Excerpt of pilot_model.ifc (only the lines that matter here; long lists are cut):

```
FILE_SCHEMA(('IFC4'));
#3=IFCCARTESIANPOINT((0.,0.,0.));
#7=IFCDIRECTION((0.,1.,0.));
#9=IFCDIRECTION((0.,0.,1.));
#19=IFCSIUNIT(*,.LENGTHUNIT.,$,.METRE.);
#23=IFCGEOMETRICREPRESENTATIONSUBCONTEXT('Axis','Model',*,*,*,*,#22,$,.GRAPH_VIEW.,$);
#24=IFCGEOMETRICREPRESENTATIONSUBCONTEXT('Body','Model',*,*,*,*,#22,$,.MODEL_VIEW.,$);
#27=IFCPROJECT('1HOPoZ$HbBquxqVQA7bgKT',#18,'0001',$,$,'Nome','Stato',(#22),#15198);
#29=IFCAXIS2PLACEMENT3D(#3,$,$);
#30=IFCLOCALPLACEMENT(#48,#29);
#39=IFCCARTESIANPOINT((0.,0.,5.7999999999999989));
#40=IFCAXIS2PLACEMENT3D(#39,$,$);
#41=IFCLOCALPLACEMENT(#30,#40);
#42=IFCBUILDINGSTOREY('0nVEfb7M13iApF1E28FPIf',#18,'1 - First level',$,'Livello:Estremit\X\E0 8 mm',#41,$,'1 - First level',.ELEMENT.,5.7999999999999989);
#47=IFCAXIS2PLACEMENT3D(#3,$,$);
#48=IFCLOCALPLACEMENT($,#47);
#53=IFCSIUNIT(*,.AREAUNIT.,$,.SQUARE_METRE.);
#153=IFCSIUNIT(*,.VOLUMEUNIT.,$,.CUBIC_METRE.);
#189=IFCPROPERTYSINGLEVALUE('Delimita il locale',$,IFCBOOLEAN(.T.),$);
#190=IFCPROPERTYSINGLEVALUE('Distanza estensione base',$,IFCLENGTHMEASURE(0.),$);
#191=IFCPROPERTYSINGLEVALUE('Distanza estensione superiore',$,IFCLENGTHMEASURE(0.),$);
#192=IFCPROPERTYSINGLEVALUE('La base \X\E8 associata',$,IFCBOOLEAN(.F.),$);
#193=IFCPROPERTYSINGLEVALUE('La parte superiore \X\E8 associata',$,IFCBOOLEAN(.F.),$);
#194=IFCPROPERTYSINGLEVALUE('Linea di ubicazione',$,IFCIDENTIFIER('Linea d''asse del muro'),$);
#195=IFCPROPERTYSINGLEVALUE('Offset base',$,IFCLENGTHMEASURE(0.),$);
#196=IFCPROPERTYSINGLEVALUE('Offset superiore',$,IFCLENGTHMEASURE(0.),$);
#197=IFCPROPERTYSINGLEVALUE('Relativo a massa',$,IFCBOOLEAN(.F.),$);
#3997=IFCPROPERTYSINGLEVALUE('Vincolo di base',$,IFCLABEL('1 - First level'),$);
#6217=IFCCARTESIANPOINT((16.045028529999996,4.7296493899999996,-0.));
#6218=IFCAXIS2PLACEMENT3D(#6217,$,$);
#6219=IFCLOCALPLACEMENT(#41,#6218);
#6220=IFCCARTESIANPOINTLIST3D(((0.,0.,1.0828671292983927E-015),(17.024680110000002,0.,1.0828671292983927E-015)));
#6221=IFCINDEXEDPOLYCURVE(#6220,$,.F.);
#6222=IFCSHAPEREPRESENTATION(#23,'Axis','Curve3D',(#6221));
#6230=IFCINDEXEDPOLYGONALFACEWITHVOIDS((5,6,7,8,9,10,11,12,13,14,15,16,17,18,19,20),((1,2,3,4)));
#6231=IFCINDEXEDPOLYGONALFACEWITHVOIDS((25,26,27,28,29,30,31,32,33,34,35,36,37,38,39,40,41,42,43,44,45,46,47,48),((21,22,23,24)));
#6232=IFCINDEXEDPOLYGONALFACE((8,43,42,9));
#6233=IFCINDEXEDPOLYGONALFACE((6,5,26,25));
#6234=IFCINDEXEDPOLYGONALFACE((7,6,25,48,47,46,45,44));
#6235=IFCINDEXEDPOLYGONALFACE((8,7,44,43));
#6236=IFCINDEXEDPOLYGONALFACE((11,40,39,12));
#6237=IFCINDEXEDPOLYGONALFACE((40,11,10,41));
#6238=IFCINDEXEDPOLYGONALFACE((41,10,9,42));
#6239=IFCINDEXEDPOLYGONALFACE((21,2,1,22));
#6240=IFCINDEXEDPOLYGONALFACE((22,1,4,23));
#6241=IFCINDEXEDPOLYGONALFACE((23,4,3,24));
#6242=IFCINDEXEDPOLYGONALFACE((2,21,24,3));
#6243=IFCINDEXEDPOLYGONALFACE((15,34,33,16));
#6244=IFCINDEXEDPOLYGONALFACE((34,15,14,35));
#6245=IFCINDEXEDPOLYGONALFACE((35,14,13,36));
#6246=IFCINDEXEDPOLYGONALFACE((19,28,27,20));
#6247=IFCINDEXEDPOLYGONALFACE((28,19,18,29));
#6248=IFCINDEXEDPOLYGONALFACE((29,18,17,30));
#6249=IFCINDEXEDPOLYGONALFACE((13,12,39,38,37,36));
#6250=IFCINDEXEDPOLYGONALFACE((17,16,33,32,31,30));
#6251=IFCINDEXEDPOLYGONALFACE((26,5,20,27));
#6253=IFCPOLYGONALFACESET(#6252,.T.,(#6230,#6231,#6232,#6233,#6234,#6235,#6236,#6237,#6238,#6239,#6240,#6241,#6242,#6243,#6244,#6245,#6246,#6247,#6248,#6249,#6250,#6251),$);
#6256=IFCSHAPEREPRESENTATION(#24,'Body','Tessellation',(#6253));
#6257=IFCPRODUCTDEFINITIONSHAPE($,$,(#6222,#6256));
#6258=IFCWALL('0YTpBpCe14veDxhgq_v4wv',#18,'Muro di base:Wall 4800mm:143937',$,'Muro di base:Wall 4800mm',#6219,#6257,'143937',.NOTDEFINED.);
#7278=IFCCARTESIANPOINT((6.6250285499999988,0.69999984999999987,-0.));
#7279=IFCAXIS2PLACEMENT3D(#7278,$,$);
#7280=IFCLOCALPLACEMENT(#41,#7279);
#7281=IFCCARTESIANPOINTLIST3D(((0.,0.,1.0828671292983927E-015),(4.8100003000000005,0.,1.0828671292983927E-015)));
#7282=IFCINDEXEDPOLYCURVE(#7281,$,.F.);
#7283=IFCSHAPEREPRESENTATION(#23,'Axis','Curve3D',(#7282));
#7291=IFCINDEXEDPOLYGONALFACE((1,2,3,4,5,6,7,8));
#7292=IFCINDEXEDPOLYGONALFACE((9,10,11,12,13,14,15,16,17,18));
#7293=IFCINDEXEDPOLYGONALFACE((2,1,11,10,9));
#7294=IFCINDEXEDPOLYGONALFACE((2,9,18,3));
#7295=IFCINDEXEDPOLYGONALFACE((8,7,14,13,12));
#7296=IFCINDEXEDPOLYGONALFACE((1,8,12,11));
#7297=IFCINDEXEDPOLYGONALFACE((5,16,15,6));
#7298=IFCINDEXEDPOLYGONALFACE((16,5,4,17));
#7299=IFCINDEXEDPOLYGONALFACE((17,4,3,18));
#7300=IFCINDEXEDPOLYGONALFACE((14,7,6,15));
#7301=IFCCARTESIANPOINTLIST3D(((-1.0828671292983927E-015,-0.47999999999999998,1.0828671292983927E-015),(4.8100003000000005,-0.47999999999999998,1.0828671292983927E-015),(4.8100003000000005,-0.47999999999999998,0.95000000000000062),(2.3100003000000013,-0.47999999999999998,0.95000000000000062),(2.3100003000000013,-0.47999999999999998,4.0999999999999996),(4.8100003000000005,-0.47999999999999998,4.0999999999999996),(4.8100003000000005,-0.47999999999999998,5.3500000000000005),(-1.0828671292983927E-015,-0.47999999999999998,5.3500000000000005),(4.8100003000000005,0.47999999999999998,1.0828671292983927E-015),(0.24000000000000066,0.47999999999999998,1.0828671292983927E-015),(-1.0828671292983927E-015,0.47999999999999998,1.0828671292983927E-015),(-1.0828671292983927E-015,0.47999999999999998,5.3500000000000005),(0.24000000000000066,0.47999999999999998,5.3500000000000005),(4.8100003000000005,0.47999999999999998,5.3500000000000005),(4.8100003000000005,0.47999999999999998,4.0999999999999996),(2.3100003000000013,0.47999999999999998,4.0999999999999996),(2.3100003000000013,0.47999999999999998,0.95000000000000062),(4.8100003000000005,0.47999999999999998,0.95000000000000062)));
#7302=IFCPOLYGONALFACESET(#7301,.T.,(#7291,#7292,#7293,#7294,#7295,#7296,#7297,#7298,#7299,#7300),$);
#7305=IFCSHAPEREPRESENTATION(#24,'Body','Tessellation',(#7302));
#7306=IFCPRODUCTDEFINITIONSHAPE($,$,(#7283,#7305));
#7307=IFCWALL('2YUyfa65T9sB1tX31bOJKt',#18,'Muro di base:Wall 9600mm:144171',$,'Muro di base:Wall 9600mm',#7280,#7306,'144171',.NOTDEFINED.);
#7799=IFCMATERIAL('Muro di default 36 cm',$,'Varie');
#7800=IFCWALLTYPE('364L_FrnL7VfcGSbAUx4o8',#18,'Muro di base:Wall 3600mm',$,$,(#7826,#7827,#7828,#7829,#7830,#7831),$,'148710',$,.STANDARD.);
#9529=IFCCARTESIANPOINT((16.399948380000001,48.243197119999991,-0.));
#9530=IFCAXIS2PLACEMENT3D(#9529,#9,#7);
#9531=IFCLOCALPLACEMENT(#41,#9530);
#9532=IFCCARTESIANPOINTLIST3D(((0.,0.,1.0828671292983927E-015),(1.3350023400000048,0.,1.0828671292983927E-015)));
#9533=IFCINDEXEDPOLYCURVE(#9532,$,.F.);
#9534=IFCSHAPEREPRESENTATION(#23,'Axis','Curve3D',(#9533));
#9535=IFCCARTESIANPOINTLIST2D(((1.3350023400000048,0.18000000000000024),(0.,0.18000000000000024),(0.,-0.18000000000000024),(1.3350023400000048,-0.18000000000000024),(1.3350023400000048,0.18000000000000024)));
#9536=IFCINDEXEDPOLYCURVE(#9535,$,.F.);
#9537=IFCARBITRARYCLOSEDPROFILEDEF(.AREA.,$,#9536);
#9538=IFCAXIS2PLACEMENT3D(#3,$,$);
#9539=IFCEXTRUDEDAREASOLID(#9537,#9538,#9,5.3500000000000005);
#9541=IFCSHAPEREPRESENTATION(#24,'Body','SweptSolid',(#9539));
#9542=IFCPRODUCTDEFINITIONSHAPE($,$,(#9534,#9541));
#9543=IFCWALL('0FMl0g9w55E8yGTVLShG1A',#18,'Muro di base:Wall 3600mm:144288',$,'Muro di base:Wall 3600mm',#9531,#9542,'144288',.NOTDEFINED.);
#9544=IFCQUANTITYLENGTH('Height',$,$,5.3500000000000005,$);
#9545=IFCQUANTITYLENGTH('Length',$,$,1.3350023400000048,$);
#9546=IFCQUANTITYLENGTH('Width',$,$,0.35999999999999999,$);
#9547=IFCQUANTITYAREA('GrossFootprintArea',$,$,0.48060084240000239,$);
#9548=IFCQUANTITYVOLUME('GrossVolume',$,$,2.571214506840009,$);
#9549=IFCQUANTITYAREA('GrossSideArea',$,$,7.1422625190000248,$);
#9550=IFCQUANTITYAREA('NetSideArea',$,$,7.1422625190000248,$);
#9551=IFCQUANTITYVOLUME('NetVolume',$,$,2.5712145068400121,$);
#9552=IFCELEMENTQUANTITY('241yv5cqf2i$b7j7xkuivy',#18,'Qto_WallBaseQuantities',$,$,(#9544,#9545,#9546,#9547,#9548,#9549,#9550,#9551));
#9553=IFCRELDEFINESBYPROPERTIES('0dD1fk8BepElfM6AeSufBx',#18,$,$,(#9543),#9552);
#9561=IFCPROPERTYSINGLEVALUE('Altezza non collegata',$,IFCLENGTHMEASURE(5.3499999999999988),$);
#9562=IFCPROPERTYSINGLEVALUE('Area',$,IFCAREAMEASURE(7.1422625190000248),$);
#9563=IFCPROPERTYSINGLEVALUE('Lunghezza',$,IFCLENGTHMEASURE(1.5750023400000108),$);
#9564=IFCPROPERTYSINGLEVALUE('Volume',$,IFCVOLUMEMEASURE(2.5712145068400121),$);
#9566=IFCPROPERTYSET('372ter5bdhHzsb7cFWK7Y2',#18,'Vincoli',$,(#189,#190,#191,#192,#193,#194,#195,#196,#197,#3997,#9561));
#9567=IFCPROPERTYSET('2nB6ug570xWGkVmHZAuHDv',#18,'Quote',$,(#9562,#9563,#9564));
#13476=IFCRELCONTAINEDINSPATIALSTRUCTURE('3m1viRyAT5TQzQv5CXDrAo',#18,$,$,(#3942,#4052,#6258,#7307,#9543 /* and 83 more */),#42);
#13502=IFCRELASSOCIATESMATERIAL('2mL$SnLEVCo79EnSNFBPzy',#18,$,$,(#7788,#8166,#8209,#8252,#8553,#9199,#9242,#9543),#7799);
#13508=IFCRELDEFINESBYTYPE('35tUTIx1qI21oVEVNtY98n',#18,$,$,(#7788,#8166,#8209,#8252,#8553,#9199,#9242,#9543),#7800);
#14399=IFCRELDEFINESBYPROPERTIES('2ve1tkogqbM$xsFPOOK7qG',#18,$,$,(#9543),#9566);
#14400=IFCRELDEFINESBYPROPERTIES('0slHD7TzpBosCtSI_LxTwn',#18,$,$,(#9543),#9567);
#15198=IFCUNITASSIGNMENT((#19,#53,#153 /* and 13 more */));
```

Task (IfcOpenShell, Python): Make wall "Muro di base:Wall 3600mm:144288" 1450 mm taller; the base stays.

```python
import ifcopenshell
import ifcopenshell.api.pset
import ifcopenshell.geom
import ifcopenshell.util.element
import ifcopenshell.util.representation
import ifcopenshell.util.shape
import ifcopenshell.util.unit

model = ifcopenshell.open("pilot_model.ifc")
unit_scale = ifcopenshell.util.unit.calculate_unit_scale(model)
area_scale = ifcopenshell.util.unit.calculate_unit_scale(model, "AREAUNIT")
volume_scale = ifcopenshell.util.unit.calculate_unit_scale(model, "VOLUMEUNIT")
settings = ifcopenshell.geom.settings()


def volume(element):
    """Net volume in cubic metres, openings subtracted."""
    shape = ifcopenshell.geom.create_shape(settings, element)
    return ifcopenshell.util.shape.get_volume(shape.geometry)


wall = model.by_guid("0FMl0g9w55E8yGTVLShG1A")
before = volume(wall)

body = ifcopenshell.util.representation.get_representation(wall, "Model", "Body")
solid = body.Items[0]
old_height = solid.Depth
solid.Depth += 1.45
after = volume(wall)
thickness = 0.36  # wall thickness in metres

# Update the stored height, areas and volumes.
qto = model.by_id(ifcopenshell.util.element.get_pset(wall, "Qto_WallBaseQuantities", should_inherit=False)["id"])
ifcopenshell.api.pset.edit_qto(model, qto=qto, properties={
    "Height": solid.Depth,
    "GrossVolume": ifcopenshell.util.element.get_pset(wall, "Qto_WallBaseQuantities", "GrossVolume") * solid.Depth / old_height,
    "GrossSideArea": ifcopenshell.util.element.get_pset(wall, "Qto_WallBaseQuantities", "GrossSideArea") * solid.Depth / old_height,
    "NetSideArea": after / thickness / area_scale,
    "NetVolume": after / volume_scale,
})
pset = model.by_id(ifcopenshell.util.element.get_pset(wall, "Vincoli", should_inherit=False)["id"])
ifcopenshell.api.pset.edit_pset(model, pset=pset, properties={
    "Altezza non collegata": model.create_entity("IfcLengthMeasure", solid.Depth),
})
pset = model.by_id(ifcopenshell.util.element.get_pset(wall, "Quote", should_inherit=False)["id"])
ifcopenshell.api.pset.edit_pset(model, pset=pset, properties={
    "Area": model.create_entity("IfcAreaMeasure", after / thickness / area_scale),
    "Volume": model.create_entity("IfcVolumeMeasure", after / volume_scale),
})

print(f"height {old_height:g} -> {solid.Depth:g}, volume {before:.3f} -> {after:.3f} m3")

model.write("pilot_model_updated.ifc")
```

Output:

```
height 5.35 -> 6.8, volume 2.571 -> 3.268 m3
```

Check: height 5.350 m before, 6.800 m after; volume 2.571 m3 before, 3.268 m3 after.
